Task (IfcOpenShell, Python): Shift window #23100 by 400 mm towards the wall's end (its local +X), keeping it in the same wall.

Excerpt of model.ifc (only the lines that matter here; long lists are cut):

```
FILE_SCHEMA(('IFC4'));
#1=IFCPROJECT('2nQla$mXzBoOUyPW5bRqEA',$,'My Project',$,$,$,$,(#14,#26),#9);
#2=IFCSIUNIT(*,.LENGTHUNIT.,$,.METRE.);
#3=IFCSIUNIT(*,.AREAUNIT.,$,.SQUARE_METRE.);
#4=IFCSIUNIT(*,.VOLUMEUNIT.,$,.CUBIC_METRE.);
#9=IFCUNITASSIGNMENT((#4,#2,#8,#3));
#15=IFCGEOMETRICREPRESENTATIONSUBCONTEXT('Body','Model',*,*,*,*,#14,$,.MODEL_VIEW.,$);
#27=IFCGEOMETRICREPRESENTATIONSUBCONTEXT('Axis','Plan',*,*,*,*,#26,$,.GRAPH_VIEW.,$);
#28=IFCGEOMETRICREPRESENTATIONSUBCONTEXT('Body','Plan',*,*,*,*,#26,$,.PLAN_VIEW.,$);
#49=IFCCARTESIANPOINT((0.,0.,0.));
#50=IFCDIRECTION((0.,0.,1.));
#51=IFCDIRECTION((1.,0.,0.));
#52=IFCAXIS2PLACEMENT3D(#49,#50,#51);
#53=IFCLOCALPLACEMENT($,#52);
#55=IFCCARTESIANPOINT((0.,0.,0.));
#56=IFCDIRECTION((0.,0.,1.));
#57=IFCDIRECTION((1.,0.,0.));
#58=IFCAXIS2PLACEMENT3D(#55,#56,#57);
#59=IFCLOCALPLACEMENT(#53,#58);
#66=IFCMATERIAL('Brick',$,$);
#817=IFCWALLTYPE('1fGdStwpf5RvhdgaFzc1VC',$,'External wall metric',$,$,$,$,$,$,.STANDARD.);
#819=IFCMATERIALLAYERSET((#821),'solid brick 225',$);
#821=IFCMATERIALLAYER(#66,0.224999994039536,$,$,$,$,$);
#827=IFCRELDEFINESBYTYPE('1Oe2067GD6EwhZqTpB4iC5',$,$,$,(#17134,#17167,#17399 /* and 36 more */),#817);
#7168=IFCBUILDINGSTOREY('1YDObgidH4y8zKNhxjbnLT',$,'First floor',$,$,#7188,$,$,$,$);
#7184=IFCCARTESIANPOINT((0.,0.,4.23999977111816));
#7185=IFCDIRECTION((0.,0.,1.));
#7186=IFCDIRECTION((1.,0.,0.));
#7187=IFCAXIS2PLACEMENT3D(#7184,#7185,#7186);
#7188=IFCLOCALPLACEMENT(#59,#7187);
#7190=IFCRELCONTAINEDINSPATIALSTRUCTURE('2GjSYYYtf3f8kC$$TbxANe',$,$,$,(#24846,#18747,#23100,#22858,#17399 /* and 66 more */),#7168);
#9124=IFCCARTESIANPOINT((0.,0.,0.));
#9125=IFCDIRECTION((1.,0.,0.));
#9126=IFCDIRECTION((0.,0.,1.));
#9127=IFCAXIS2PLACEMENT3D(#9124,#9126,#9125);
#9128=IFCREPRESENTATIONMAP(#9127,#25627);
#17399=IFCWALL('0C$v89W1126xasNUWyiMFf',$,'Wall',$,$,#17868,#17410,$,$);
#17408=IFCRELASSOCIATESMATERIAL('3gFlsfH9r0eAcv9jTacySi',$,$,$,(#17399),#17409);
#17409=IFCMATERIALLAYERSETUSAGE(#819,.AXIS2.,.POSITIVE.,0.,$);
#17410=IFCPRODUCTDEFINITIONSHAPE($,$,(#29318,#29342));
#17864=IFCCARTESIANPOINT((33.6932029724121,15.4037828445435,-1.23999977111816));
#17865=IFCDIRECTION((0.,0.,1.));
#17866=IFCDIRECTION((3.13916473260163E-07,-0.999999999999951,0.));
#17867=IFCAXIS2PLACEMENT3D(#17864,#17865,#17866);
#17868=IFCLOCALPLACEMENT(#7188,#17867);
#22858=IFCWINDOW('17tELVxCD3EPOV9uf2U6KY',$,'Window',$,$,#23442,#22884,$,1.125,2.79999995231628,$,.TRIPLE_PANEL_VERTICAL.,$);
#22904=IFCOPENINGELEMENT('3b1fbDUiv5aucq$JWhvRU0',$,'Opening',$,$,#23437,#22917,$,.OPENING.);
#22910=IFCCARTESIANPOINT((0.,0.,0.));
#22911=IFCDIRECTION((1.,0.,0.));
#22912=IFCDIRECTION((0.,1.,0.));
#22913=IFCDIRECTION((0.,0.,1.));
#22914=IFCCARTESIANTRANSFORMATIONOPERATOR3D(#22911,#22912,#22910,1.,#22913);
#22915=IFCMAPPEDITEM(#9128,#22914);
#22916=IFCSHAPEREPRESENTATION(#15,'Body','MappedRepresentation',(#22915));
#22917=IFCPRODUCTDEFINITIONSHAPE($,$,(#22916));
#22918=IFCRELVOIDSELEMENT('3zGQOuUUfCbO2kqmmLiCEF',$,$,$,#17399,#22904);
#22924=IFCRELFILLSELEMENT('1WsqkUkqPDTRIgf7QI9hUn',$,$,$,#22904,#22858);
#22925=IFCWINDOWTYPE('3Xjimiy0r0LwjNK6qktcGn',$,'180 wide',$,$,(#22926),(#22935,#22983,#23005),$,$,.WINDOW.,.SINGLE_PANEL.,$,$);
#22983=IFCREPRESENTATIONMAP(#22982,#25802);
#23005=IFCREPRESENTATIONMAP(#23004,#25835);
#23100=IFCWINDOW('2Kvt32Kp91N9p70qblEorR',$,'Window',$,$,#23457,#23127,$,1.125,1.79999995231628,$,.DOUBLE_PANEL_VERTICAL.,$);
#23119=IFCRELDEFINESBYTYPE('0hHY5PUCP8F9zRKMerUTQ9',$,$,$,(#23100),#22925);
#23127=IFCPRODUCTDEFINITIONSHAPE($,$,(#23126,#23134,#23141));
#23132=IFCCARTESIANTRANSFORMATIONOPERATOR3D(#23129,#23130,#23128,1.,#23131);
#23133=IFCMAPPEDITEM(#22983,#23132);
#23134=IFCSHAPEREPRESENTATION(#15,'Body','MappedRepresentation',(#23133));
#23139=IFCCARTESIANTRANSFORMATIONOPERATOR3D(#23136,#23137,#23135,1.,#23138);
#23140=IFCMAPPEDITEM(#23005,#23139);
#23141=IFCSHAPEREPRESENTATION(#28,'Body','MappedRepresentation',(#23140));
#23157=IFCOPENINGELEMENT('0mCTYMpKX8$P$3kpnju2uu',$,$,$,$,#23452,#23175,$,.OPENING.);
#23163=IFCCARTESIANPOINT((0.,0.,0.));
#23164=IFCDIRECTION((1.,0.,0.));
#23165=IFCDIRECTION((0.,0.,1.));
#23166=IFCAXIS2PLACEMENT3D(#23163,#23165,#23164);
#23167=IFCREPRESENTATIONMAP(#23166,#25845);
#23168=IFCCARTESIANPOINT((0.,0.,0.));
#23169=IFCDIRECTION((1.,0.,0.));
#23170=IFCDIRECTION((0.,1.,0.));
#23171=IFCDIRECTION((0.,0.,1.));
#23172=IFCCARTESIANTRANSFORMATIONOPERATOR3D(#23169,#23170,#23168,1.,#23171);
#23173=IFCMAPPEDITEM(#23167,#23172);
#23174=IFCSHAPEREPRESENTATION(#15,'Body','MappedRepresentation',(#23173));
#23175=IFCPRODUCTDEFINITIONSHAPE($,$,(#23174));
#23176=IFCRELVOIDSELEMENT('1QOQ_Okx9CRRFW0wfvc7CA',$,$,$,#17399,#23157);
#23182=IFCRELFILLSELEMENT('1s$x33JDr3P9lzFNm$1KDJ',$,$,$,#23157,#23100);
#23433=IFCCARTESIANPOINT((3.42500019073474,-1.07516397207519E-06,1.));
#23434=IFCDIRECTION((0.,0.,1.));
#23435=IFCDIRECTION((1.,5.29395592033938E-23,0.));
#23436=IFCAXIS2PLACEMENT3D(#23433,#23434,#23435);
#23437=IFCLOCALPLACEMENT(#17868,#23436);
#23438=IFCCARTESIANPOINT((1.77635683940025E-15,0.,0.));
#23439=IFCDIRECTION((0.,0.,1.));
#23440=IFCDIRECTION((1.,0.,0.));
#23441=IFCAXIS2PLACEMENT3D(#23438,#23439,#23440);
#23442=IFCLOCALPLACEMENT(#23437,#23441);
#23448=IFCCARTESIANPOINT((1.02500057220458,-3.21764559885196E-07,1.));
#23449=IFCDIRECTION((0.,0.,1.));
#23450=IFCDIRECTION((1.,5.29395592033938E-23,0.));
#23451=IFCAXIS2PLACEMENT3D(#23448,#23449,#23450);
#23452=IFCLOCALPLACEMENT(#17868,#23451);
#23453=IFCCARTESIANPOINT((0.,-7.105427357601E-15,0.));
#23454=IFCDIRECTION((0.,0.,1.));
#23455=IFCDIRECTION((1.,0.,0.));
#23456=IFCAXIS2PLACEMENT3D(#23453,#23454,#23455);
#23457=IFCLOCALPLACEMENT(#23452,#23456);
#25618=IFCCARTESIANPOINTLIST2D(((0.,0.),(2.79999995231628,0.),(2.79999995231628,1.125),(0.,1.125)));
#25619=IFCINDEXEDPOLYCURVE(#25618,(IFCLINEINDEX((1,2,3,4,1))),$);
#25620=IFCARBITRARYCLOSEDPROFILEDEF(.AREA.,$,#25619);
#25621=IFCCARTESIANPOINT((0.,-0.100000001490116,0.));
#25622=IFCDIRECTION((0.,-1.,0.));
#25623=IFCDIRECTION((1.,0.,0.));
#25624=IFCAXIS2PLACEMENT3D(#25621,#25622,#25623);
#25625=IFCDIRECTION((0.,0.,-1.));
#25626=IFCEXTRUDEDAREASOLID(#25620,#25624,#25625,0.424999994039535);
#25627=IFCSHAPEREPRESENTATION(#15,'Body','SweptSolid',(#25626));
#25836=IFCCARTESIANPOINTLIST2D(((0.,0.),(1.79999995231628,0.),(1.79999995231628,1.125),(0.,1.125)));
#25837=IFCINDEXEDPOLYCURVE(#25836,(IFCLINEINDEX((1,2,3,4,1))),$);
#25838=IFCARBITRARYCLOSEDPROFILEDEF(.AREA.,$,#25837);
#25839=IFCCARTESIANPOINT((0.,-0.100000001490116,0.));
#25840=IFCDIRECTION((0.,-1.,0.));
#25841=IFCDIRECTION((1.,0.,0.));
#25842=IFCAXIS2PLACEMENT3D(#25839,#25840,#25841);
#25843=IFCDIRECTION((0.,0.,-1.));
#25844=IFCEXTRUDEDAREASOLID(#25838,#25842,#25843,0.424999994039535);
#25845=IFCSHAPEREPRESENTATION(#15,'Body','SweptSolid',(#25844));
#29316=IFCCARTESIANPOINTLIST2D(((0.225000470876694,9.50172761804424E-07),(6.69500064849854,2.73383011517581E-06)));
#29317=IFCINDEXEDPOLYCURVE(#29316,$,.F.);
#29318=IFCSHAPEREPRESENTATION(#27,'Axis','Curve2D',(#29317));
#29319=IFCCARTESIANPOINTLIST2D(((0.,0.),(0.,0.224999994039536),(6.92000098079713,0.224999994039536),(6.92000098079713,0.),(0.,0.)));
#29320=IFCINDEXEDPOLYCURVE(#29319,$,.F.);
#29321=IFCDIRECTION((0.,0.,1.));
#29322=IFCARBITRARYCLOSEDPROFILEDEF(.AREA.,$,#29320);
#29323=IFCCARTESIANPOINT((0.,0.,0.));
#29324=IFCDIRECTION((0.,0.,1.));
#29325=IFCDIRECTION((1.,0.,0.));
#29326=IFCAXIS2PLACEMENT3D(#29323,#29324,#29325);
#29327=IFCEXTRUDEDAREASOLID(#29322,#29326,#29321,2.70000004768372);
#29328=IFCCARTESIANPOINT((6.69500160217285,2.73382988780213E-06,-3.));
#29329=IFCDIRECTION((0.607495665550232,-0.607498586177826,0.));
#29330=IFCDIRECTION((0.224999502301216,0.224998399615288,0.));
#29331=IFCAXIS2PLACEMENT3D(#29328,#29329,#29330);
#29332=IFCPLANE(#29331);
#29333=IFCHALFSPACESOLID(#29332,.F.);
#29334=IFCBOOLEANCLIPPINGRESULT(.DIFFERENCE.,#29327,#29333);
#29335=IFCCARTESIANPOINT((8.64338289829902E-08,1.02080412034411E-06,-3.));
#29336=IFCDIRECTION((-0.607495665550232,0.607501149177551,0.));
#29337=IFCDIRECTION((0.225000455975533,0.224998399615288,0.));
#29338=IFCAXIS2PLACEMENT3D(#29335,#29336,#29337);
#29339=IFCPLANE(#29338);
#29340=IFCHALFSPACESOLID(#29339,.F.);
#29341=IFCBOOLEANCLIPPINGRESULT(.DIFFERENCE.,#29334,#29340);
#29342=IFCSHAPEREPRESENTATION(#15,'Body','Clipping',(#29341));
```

```python
import ifcopenshell
import ifcopenshell.api.geometry
import ifcopenshell.util.placement
import ifcopenshell.util.unit

model = ifcopenshell.open("model.ifc")
unit_scale = ifcopenshell.util.unit.calculate_unit_scale(model)

window = model.by_guid("2Kvt32Kp91N9p70qblEorR")
opening = window.FillsVoids[0].RelatingOpeningElement
wall = opening.VoidsElements[0].RelatingBuildingElement

wall_matrix = ifcopenshell.util.placement.get_local_placement(wall.ObjectPlacement)
shift = wall_matrix[:3, 0] * 0.4 / unit_scale
before = ifcopenshell.util.placement.get_local_placement(window.ObjectPlacement)[:3, 3].copy()

# The window is placed relative to its opening, so it follows when the opening moves.
matrix = ifcopenshell.util.placement.get_local_placement(opening.ObjectPlacement)
matrix[:3, 3] += shift
ifcopenshell.api.geometry.edit_object_placement(
    model, product=opening, matrix=matrix, is_si=False, should_transform_children=True
)

after = ifcopenshell.util.placement.get_local_placement(window.ObjectPlacement)[:3, 3]
print("window moved by", (after - before).round(3) + 0.0)

model.write("model_v2.ifc")
```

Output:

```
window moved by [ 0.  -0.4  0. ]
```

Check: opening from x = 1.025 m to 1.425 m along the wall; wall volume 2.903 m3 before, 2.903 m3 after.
